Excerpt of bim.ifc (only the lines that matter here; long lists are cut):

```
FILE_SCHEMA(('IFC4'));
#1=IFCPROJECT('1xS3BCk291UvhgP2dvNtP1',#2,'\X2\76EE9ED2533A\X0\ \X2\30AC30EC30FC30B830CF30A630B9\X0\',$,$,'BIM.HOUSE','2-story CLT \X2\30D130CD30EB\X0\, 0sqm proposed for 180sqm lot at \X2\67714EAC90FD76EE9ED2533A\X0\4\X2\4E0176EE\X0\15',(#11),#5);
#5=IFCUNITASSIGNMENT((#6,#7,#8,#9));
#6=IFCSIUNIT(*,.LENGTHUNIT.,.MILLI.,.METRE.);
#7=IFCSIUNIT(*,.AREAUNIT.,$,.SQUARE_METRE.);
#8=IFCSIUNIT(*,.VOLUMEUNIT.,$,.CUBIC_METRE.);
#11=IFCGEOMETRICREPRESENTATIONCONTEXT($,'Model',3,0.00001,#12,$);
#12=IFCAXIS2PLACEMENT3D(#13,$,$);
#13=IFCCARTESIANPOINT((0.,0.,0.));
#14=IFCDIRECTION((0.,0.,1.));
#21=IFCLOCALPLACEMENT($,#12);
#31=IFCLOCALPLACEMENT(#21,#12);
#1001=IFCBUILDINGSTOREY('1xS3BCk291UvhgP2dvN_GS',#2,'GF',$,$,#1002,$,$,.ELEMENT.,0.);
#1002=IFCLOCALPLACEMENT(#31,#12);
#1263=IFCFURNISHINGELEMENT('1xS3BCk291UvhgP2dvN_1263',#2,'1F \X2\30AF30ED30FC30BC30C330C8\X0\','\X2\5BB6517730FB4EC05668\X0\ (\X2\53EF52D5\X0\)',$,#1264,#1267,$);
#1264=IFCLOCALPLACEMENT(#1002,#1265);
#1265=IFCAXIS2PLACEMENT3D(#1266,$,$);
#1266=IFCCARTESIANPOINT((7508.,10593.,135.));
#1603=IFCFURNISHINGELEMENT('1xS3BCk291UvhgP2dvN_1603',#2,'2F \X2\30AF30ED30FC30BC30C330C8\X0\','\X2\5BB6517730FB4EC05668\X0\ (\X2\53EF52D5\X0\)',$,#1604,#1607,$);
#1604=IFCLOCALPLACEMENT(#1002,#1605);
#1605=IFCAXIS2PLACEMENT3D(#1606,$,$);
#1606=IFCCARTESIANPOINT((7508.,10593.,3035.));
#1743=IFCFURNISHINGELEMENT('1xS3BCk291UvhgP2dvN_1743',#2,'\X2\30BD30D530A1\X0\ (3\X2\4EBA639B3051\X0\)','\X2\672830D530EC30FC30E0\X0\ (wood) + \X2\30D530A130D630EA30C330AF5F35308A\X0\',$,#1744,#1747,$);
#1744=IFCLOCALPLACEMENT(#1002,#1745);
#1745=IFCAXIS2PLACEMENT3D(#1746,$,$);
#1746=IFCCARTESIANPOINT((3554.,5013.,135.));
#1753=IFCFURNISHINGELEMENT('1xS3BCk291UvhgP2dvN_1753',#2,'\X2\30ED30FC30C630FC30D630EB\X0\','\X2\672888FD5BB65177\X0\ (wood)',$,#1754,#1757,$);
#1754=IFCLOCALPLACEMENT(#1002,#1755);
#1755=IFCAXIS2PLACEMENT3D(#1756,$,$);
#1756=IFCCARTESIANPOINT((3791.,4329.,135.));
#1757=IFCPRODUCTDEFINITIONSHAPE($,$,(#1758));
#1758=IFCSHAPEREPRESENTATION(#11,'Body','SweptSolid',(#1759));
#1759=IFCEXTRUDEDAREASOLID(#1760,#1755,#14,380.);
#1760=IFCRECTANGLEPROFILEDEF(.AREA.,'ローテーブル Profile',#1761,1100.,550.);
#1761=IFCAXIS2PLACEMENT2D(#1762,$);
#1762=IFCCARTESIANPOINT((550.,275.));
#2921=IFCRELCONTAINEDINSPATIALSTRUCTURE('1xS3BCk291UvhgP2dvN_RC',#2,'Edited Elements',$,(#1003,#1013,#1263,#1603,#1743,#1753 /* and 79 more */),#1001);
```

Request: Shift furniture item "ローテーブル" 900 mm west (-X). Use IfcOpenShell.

```python
import ifcopenshell
import ifcopenshell.api.geometry
import ifcopenshell.util.placement
import ifcopenshell.util.unit

model = ifcopenshell.open("bim.ifc")
unit_scale = ifcopenshell.util.unit.calculate_unit_scale(model)

item = model.by_guid("1xS3BCk291UvhgP2dvN_1753")
matrix = ifcopenshell.util.placement.get_local_placement(item.ObjectPlacement)
matrix[0, 3] -= 0.9 / unit_scale
ifcopenshell.api.geometry.edit_object_placement(model, product=item, matrix=matrix, is_si=False)

print(ifcopenshell.util.placement.get_local_placement(item.ObjectPlacement).round(3) + 0.0)

model.write("bim_edited.ifc")
```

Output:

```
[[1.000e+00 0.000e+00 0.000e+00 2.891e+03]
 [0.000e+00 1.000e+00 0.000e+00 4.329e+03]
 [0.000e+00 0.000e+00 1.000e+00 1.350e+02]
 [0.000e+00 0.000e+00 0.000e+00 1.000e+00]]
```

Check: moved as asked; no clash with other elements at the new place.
